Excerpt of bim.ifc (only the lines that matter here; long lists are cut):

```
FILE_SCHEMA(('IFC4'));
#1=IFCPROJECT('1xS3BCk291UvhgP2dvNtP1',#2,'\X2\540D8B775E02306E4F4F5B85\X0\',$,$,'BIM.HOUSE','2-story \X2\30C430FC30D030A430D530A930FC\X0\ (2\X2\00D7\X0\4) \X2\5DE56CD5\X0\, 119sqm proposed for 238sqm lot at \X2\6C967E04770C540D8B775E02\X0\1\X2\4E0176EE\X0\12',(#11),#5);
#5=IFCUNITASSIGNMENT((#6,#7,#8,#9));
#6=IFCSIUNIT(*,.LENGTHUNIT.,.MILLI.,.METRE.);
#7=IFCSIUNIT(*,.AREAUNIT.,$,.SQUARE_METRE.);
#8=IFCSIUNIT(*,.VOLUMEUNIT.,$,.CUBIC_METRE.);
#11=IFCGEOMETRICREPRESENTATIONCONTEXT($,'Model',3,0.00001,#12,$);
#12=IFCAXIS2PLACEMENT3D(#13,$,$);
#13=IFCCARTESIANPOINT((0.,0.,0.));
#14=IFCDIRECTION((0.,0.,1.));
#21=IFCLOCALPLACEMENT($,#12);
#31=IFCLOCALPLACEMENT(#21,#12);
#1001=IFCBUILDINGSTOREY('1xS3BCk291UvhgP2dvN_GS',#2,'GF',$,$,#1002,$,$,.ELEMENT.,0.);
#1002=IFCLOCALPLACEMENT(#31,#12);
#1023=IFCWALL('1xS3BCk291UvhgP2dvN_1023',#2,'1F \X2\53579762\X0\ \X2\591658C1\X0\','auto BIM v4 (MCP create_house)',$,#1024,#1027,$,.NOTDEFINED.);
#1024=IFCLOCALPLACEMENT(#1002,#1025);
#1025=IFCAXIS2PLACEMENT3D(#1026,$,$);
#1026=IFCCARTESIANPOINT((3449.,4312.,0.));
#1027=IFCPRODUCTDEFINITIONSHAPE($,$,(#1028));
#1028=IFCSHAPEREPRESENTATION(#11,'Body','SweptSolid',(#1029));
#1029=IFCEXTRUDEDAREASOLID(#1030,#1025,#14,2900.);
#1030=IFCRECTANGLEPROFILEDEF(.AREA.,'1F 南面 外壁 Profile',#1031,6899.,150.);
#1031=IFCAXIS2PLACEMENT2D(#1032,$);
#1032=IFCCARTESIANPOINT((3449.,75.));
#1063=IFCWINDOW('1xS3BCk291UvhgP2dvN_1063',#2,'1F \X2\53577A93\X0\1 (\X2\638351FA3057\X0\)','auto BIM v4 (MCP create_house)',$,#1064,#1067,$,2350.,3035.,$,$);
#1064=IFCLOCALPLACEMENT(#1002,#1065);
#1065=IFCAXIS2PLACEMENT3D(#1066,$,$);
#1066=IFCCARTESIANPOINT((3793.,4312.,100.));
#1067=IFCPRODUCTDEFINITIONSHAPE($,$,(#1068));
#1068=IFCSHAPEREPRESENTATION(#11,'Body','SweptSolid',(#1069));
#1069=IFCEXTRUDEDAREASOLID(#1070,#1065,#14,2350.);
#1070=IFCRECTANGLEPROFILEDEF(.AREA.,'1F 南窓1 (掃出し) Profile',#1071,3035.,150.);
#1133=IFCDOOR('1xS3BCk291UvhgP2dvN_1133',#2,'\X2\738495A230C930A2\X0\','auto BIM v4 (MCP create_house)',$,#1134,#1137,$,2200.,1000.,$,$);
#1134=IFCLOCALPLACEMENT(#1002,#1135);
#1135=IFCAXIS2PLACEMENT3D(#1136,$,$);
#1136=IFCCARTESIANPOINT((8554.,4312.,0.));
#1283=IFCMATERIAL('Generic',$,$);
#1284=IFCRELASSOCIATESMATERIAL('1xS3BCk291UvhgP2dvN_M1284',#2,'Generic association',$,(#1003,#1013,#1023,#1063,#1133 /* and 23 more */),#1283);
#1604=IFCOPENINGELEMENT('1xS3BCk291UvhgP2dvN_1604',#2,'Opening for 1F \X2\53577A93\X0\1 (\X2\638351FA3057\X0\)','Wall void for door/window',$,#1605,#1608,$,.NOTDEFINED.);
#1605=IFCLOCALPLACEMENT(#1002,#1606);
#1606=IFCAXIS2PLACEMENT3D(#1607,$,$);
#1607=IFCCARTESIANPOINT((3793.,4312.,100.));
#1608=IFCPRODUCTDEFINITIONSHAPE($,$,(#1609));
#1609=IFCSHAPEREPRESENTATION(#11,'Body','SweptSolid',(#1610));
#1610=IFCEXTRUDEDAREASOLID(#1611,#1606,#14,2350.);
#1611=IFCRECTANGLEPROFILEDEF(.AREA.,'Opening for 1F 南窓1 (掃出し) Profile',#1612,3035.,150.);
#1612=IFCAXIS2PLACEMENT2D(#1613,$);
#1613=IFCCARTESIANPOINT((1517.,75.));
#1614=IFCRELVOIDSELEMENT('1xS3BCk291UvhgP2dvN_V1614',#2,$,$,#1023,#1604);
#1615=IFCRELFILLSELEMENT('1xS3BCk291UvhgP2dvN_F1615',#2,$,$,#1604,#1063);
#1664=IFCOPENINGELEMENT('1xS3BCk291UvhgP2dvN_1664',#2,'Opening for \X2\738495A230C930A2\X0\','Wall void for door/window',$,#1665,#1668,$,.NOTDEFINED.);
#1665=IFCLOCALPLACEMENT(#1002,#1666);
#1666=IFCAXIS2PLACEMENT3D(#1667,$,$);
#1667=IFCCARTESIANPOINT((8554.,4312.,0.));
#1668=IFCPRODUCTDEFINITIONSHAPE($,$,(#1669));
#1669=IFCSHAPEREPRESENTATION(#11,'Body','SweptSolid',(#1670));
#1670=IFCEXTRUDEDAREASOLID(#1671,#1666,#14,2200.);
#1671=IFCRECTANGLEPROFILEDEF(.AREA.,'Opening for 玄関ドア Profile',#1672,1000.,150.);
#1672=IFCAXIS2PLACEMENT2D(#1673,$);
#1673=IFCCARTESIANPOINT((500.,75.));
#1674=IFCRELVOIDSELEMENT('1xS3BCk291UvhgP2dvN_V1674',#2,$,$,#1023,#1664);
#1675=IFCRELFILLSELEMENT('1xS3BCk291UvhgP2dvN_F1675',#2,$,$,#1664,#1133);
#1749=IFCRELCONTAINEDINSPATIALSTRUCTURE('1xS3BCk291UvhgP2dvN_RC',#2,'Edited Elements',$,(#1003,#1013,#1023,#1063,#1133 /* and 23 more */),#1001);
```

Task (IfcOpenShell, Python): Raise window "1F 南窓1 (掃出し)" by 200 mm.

```python
import numpy as np
import ifcopenshell
import ifcopenshell.api.geometry
import ifcopenshell.util.placement
import ifcopenshell.util.unit

model = ifcopenshell.open("bim.ifc")
unit_scale = ifcopenshell.util.unit.calculate_unit_scale(model)

window = model.by_guid("1xS3BCk291UvhgP2dvN_1063")
opening = window.FillsVoids[0].RelatingOpeningElement
dz = 0.2 / unit_scale

shift = np.array([0.0, 0.0, dz])
# The window is not placed relative to its opening, so move both.
for product in (opening, window):
    matrix = ifcopenshell.util.placement.get_local_placement(product.ObjectPlacement)
    matrix[:3, 3] += shift
    ifcopenshell.api.geometry.edit_object_placement(model, product=product, matrix=matrix, is_si=False)

print(f"moved by {dz * unit_scale:+.3f} m")

model.write("bim-out.ifc")
```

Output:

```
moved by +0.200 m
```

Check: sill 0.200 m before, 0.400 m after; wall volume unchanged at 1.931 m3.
